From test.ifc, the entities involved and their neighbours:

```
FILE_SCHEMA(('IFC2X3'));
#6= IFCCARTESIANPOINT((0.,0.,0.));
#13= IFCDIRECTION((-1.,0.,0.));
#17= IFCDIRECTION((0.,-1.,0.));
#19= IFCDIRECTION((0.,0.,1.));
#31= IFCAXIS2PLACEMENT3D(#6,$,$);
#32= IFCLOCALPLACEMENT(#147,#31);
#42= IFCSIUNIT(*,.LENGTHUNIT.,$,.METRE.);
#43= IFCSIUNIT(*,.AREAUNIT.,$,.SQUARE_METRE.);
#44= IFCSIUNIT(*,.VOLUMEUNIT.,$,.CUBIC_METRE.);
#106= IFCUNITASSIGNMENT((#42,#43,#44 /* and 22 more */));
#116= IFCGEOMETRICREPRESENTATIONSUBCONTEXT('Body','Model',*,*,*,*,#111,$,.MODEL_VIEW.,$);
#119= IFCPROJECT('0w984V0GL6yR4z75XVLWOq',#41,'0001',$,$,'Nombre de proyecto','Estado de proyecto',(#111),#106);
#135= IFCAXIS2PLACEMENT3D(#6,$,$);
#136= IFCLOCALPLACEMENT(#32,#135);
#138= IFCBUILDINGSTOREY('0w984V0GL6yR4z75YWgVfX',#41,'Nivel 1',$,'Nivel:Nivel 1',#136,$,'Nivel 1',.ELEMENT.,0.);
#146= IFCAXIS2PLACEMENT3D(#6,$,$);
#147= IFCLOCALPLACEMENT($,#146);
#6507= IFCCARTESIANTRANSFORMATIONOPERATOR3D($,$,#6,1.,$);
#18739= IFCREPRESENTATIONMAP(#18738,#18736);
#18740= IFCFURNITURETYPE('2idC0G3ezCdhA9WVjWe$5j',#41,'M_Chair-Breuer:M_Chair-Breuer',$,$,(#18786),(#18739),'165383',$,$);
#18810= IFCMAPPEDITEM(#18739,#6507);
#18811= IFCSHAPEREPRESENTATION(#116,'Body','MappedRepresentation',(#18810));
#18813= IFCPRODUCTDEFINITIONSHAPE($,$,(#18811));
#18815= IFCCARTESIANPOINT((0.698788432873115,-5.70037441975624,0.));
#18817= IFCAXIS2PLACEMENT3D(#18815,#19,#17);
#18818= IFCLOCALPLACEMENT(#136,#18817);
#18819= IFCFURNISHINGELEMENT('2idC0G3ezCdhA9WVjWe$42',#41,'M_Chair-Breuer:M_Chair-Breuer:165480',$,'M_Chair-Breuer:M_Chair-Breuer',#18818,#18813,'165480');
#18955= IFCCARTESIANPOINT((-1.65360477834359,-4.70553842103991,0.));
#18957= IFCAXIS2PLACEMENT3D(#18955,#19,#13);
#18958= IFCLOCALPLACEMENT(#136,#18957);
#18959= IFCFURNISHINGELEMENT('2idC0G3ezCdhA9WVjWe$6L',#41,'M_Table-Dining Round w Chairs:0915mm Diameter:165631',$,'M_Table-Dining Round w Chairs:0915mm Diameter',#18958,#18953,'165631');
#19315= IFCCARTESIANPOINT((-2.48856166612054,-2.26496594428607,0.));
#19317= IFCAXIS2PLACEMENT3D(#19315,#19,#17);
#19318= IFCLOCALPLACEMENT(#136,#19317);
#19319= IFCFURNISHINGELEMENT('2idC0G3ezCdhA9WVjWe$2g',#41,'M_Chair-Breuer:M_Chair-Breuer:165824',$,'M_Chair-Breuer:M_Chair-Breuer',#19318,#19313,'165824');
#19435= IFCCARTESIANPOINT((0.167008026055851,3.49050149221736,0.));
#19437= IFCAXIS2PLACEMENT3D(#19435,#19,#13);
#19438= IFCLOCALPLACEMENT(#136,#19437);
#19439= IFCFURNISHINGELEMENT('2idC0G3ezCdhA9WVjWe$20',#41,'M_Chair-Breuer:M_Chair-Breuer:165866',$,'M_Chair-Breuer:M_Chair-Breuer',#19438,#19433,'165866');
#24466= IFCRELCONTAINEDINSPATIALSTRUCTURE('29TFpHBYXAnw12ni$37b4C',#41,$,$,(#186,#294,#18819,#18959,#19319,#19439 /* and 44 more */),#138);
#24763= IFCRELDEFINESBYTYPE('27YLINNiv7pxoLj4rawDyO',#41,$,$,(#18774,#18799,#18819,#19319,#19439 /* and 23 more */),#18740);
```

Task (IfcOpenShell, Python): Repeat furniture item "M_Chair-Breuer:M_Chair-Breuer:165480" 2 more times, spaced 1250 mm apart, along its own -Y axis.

```python
import ifcopenshell
import ifcopenshell.api.geometry
import ifcopenshell.api.root
import ifcopenshell.util.element
import ifcopenshell.util.placement
import ifcopenshell.util.unit

model = ifcopenshell.open("test.ifc")
unit_scale = ifcopenshell.util.unit.calculate_unit_scale(model)


def reuse_history(source, copy):
    """copy_class also copies each property set's owner history, people and application; keep the originals."""
    for rel in copy.IsDefinedBy:
        if rel.is_a("IfcRelDefinesByProperties") and (history := rel.RelatingPropertyDefinition.OwnerHistory):
            rel.RelatingPropertyDefinition.OwnerHistory = source.OwnerHistory
            ifcopenshell.util.element.remove_deep2(model, history)


source = model.by_id(18819)
base = ifcopenshell.util.placement.get_local_placement(source.ObjectPlacement)
step = -base[:3, 1] * 1.25 / unit_scale

for i in range(1, 3):
    copy = ifcopenshell.api.root.copy_class(model, product=source)
    copy.Representation = ifcopenshell.util.element.copy_deep(
        model, source.Representation, exclude=["IfcGeometricRepresentationContext", "IfcRepresentationMap"]
    )
    copy.Name = "M_Chair-Breuer:M_Chair-Breuer"
    copy.Tag = None
    reuse_history(source, copy)
    matrix = base.copy()
    matrix[:3, 3] += i * step
    print("added at", matrix[:3, 3].round(3) + 0.0)
    ifcopenshell.api.geometry.edit_object_placement(model, product=copy, matrix=matrix, is_si=False)

model.write("test-out.ifc")
```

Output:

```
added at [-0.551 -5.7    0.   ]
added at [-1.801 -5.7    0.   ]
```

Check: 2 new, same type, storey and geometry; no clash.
